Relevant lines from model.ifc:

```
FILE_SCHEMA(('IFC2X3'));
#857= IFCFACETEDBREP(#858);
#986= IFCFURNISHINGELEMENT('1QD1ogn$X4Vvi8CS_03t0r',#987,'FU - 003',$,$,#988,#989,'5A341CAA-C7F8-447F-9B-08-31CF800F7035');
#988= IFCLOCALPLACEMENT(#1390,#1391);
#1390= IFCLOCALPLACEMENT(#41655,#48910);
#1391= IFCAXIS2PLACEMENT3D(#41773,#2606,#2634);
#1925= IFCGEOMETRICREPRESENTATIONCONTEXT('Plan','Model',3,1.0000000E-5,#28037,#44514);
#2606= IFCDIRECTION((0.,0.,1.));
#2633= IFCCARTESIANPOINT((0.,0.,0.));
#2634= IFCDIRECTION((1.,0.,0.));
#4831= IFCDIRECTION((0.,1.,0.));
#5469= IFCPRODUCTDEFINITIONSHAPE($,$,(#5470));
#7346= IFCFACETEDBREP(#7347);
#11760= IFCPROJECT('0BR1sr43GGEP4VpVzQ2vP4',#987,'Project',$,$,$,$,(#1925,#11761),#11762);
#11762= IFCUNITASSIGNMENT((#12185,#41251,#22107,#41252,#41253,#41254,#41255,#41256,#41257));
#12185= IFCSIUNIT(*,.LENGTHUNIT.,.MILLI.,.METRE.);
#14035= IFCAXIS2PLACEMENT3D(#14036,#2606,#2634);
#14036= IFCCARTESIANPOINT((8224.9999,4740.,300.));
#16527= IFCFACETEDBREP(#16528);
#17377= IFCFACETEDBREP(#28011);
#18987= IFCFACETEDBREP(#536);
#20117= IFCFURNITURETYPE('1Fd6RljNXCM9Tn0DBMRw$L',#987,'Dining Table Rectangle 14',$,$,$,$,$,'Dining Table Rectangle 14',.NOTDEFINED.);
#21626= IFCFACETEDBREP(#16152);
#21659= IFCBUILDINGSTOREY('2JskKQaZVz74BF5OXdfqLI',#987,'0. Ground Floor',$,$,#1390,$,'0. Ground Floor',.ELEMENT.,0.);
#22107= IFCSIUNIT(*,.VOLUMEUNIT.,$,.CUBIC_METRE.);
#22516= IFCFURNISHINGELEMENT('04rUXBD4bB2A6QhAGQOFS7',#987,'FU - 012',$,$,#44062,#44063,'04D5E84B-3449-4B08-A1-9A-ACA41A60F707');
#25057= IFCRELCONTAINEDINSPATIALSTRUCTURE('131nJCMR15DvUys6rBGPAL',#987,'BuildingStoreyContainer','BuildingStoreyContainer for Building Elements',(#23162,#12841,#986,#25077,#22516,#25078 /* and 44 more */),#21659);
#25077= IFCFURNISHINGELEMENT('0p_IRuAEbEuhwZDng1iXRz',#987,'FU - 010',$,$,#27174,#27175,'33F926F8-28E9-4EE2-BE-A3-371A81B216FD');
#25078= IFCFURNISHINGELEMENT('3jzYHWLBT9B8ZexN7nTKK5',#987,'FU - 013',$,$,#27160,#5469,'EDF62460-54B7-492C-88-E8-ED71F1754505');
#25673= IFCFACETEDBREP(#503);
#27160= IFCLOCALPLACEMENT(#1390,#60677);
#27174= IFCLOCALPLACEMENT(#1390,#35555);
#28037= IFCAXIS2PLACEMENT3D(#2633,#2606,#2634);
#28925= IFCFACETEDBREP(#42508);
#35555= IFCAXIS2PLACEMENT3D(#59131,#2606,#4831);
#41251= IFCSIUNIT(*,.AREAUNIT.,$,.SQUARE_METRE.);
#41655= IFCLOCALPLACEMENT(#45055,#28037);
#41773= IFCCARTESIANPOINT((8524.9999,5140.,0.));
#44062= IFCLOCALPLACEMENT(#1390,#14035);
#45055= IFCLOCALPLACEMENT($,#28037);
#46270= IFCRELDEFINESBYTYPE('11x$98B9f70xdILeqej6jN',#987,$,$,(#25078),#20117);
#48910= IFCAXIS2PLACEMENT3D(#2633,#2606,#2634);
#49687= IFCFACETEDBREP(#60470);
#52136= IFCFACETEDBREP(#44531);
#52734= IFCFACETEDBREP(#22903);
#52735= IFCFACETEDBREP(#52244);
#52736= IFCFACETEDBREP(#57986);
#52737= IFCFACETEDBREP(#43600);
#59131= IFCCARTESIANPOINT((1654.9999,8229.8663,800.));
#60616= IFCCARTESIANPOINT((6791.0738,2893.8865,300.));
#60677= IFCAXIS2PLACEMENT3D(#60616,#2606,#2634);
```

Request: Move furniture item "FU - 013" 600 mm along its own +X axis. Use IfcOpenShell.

```python
import ifcopenshell
import ifcopenshell.api.geometry
import ifcopenshell.util.placement
import ifcopenshell.util.unit

model = ifcopenshell.open("model.ifc")
unit_scale = ifcopenshell.util.unit.calculate_unit_scale(model)

item = model.by_guid("3jzYHWLBT9B8ZexN7nTKK5")
matrix = ifcopenshell.util.placement.get_local_placement(item.ObjectPlacement)
matrix[:3, 3] += matrix[:3, 0] * 0.6 / unit_scale
ifcopenshell.api.geometry.edit_object_placement(model, product=item, matrix=matrix, is_si=False)

print(ifcopenshell.util.placement.get_local_placement(item.ObjectPlacement).round(3) + 0.0)

model.write("model-out.ifc")
```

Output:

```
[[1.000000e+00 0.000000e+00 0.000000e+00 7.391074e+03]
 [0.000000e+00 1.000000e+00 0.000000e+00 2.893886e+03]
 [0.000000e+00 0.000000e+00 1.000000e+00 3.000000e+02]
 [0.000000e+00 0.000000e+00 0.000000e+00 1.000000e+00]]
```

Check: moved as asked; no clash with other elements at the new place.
